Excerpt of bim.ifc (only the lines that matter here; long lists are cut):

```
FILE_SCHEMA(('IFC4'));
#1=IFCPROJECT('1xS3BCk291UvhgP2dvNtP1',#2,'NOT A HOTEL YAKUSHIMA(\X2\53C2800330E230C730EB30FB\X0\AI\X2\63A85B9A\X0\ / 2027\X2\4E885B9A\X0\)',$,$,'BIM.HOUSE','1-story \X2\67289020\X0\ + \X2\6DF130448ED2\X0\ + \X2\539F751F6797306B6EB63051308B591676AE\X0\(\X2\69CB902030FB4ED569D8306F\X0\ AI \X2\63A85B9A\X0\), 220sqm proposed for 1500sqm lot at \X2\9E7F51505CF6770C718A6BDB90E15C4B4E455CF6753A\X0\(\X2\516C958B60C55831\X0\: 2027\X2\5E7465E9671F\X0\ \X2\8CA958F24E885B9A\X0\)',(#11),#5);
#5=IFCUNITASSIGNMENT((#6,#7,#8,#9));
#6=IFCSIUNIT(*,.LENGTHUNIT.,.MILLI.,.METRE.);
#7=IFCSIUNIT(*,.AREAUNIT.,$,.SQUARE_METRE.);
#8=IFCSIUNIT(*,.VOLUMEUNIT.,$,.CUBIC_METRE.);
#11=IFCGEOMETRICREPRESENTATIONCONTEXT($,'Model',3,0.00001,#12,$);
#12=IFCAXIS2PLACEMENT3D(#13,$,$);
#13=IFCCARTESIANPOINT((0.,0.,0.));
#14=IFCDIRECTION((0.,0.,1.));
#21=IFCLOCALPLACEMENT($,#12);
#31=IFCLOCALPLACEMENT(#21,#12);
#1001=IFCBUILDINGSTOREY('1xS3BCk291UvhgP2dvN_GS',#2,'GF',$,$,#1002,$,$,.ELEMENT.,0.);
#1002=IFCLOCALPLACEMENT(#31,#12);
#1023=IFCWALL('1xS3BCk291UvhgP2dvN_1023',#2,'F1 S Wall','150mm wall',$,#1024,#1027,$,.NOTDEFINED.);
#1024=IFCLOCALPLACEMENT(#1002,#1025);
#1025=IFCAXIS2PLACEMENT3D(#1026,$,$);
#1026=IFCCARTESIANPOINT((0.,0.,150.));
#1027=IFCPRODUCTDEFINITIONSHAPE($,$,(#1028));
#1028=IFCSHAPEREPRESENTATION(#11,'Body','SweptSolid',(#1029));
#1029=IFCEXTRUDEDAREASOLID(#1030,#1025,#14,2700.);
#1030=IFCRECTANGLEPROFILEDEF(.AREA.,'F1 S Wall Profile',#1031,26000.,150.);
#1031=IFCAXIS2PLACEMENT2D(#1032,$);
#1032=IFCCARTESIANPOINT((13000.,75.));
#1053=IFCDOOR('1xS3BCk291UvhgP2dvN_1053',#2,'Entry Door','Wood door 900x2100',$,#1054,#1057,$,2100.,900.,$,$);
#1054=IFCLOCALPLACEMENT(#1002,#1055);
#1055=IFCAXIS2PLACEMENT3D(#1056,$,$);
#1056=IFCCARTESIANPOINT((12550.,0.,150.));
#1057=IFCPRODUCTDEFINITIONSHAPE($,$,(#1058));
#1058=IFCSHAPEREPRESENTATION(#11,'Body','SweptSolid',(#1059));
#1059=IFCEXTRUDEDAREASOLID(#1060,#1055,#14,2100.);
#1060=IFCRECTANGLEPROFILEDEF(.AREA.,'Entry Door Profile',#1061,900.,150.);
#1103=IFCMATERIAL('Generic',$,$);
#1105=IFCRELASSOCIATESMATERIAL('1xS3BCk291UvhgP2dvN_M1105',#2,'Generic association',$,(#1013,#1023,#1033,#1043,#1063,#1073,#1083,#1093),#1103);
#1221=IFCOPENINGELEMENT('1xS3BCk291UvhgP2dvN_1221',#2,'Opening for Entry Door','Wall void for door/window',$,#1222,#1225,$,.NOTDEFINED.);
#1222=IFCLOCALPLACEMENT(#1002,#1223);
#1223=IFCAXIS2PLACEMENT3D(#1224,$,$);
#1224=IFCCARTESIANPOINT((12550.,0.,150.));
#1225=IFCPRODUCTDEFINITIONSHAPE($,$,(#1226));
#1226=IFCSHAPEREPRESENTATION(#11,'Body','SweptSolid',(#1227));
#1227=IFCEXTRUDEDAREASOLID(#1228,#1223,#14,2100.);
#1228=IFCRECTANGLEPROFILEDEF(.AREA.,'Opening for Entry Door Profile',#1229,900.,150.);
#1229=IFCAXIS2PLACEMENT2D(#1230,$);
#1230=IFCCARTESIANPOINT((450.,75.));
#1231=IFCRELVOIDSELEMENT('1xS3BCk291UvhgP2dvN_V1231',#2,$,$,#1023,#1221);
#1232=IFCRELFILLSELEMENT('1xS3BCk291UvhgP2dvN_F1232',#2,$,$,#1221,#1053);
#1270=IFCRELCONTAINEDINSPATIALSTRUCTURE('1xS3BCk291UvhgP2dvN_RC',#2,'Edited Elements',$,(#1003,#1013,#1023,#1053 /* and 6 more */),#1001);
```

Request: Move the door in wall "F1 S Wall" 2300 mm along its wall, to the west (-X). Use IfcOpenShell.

```python
import ifcopenshell
import ifcopenshell.api.geometry
import ifcopenshell.util.placement
import ifcopenshell.util.unit

model = ifcopenshell.open("bim.ifc")
unit_scale = ifcopenshell.util.unit.calculate_unit_scale(model)

door = model.by_guid("1xS3BCk291UvhgP2dvN_1053")
opening = door.FillsVoids[0].RelatingOpeningElement
wall = opening.VoidsElements[0].RelatingBuildingElement

wall_matrix = ifcopenshell.util.placement.get_local_placement(wall.ObjectPlacement)
shift = wall_matrix[:3, 0] * -2.3 / unit_scale
before = ifcopenshell.util.placement.get_local_placement(door.ObjectPlacement)[:3, 3].copy()

# The door is not placed relative to its opening, so move both.
for product in (opening, door):
    matrix = ifcopenshell.util.placement.get_local_placement(product.ObjectPlacement)
    matrix[:3, 3] += shift
    ifcopenshell.api.geometry.edit_object_placement(model, product=product, matrix=matrix, is_si=False)

after = ifcopenshell.util.placement.get_local_placement(door.ObjectPlacement)[:3, 3]
print("door moved by", (after - before).round(3) + 0.0)

model.write("bim_v2.ifc")
```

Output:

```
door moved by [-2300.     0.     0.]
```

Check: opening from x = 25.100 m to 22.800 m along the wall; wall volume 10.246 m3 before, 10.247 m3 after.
